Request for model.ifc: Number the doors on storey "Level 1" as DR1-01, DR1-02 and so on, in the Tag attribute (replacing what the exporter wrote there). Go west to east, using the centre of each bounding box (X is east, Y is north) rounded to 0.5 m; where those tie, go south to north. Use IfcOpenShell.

First a look at what the model holds.

```python
import ifcopenshell
import ifcopenshell.util.element
import ifcopenshell.util.placement

model = ifcopenshell.open("model.ifc")
print(model.schema)
storey = next(s for s in model.by_type("IfcBuildingStorey") if s.Name == "Level 1")
doors = [e for e in ifcopenshell.util.element.get_decomposition(storey) if e.is_a("IfcDoor")]
for e in sorted(doors, key=lambda e: e.id()):
    origin = ifcopenshell.util.placement.get_local_placement(e.ObjectPlacement)[:3, 3]
    print(e.id(), e.Tag, e.Name, origin.round(2) + 0.0, sep=" | ")
```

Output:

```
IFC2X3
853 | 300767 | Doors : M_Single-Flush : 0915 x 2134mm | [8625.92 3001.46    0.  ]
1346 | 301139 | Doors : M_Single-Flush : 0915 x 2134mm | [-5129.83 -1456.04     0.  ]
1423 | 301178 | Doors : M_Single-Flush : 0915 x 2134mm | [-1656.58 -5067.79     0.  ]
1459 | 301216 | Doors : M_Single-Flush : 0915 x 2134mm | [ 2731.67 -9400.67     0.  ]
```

```python
import ifcopenshell
import ifcopenshell.geom
import ifcopenshell.util.element
import ifcopenshell.util.shape

model = ifcopenshell.open("model.ifc")
settings = ifcopenshell.geom.settings()
settings.set("use-world-coords", True)


def centre(element):
    shape = ifcopenshell.geom.create_shape(settings, element)
    return ifcopenshell.util.shape.get_bbox_centroid(shape.geometry)


storey = next(s for s in model.by_type("IfcBuildingStorey") if s.Name == "Level 1")
doors = [e for e in ifcopenshell.util.element.get_decomposition(storey) if e.is_a("IfcDoor")]

# Insertion points can sit at a corner or the storey origin, so sort by the geometry (in metres).
centres = {e: centre(e) for e in doors}
doors.sort(key=lambda e: (round(centres[e][0] / 0.5), centres[e][1]))

for i, e in enumerate(doors, start=1):
    number = f"DR1-{i:02d}"
    e.Tag = number
    print(e.id(), number)

model.write("model-out.ifc")
```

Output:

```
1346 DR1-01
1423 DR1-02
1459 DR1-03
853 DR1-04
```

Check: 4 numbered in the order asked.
